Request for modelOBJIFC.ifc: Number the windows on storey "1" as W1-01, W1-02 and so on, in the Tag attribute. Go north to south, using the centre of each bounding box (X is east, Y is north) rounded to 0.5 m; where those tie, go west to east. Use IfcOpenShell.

First a look at what the model holds.

```python
import ifcopenshell
import ifcopenshell.util.element
import ifcopenshell.util.placement

model = ifcopenshell.open("modelOBJIFC.ifc")
print(model.schema)
storey = next(s for s in model.by_type("IfcBuildingStorey") if s.Name == "1")
windows = [e for e in ifcopenshell.util.element.get_decomposition(storey) if e.is_a("IfcWindow")]
for e in sorted(windows, key=lambda e: e.id()):
    origin = ifcopenshell.util.placement.get_local_placement(e.ObjectPlacement)[:3, 3]
    print(e.id(), e.Tag, e.Name, origin.round(2) + 0.0, sep=" | ")
```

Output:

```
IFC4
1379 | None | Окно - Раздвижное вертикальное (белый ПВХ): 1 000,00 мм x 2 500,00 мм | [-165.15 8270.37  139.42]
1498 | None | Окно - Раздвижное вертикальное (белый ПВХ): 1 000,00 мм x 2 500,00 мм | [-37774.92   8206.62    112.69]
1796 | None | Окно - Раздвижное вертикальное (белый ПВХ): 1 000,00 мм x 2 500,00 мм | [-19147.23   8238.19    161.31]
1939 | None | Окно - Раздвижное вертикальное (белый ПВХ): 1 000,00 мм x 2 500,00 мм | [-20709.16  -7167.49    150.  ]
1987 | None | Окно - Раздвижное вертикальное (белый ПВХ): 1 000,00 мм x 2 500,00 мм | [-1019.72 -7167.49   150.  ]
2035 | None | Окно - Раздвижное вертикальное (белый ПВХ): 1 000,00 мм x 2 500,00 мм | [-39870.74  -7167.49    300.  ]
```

```python
import ifcopenshell
import ifcopenshell.geom
import ifcopenshell.util.element
import ifcopenshell.util.shape

model = ifcopenshell.open("modelOBJIFC.ifc")
settings = ifcopenshell.geom.settings()
settings.set("use-world-coords", True)


def centre(element):
    shape = ifcopenshell.geom.create_shape(settings, element)
    return ifcopenshell.util.shape.get_bbox_centroid(shape.geometry)


storey = next(s for s in model.by_type("IfcBuildingStorey") if s.Name == "1")
windows = [e for e in ifcopenshell.util.element.get_decomposition(storey) if e.is_a("IfcWindow")]

# Insertion points can sit at a corner or the storey origin, so sort by the geometry (in metres).
centres = {e: centre(e) for e in windows}
windows.sort(key=lambda e: (-round(centres[e][1] / 0.5), centres[e][0]))

for i, e in enumerate(windows, start=1):
    number = f"W1-{i:02d}"
    e.Tag = number
    print(e.id(), number)

model.write("modelOBJIFC_edited.ifc")
```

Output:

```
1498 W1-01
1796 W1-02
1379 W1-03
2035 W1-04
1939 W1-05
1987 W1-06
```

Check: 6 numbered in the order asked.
